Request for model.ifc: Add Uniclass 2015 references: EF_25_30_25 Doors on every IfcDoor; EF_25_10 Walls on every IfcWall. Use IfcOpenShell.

First a look at what the model holds.

```python
import ifcopenshell

model = ifcopenshell.open("model.ifc")
print(model.schema)
print("classifications:", [c.Name for c in model.by_type("IfcClassification")])
for ifc_class in ("IfcDoor", "IfcRoof", "IfcStair", "IfcWall", "IfcWindow"):
    print(ifc_class, len(model.by_type(ifc_class)))
```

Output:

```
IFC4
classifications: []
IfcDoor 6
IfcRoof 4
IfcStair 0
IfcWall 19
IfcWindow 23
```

```python
import ifcopenshell
import ifcopenshell.api.classification

model = ifcopenshell.open("model.ifc")

system = ifcopenshell.api.classification.add_classification(model, classification="Uniclass 2015")

codes = {
    "IfcDoor": ("EF_25_30_25", "Doors"),
    "IfcWall": ("EF_25_10", "Walls"),
}
for ifc_class, (code, name) in codes.items():
    products = model.by_type(ifc_class)
    ifcopenshell.api.classification.add_reference(
        model, products=products, classification=system, identification=code, name=name
    )
    print(code, len(products))

model.write("model_rev.ifc")
```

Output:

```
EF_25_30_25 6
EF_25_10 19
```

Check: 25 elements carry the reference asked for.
